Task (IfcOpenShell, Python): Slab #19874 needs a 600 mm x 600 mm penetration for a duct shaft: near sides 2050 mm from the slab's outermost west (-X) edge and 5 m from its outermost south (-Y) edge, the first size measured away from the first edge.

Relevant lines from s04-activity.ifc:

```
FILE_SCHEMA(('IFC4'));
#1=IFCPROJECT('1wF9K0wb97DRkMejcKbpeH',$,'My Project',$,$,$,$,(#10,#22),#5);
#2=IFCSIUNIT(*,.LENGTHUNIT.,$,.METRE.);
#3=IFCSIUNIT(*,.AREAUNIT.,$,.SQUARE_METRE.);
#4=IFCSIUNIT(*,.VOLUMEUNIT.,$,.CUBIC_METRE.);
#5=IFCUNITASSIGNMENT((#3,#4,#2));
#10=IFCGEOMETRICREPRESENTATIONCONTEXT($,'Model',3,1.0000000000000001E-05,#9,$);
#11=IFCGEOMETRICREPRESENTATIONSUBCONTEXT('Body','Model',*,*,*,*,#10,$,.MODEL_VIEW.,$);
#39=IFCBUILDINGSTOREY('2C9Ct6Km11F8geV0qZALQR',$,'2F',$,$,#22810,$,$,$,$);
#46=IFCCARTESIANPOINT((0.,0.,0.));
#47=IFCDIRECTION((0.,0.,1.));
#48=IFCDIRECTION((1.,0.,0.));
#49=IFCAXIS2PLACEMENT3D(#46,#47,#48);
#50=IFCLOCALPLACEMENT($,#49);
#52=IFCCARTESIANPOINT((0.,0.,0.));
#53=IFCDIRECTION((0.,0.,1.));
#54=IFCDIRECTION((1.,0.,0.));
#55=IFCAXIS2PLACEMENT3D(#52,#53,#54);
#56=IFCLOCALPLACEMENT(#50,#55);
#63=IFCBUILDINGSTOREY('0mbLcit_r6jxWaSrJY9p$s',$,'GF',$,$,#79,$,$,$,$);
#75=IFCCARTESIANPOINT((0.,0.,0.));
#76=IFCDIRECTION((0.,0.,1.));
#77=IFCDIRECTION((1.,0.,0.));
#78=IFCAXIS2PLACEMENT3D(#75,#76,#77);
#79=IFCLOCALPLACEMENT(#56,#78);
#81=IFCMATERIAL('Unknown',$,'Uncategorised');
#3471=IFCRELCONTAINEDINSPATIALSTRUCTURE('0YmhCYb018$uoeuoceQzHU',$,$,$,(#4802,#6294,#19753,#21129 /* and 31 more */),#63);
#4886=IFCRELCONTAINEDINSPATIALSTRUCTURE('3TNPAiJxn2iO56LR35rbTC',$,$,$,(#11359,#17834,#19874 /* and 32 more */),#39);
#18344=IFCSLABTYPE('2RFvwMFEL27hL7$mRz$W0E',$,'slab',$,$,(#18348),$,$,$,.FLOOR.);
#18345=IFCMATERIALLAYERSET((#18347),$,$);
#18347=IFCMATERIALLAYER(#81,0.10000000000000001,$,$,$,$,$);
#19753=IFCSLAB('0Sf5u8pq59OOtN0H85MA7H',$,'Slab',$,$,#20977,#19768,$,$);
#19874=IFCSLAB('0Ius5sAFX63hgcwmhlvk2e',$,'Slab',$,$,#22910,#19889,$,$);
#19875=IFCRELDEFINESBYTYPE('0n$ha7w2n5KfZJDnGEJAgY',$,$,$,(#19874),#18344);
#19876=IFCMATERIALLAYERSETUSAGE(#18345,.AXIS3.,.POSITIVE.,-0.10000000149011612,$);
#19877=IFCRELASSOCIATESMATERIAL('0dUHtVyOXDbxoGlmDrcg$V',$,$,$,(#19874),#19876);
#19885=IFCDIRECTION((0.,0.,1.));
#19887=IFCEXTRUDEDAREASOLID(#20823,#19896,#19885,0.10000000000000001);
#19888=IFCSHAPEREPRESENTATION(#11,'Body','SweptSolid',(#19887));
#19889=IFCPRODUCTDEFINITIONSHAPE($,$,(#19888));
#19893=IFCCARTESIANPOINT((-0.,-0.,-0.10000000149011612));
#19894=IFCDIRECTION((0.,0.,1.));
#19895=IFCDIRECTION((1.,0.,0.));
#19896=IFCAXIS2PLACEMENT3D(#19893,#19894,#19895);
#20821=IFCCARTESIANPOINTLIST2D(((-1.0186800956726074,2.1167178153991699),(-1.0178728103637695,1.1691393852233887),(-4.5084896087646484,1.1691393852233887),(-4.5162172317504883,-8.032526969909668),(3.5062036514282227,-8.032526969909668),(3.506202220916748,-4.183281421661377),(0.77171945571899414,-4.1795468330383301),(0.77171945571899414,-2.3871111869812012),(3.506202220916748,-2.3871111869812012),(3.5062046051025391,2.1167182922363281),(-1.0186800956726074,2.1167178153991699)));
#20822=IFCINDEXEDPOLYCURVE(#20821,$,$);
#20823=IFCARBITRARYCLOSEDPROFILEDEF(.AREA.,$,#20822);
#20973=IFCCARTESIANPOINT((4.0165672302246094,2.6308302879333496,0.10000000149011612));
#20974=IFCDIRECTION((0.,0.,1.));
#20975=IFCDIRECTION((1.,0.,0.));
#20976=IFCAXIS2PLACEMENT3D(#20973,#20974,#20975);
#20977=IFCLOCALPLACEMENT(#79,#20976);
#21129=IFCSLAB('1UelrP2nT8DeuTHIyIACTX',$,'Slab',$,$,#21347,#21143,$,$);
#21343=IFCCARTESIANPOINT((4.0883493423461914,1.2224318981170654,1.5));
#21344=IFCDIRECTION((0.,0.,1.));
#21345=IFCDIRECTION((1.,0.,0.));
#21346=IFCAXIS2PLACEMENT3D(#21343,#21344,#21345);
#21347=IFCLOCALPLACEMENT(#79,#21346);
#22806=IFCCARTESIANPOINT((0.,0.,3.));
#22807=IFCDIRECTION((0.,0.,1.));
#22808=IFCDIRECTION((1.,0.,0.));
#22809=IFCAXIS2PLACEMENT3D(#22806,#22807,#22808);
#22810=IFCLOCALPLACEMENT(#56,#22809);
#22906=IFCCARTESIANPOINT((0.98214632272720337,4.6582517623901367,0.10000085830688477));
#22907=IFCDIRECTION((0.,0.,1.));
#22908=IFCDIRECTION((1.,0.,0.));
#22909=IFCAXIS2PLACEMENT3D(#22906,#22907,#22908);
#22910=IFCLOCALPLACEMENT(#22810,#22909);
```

```python
import numpy as np
import ifcopenshell
import ifcopenshell.api.feature
import ifcopenshell.api.geometry
import ifcopenshell.api.root
import ifcopenshell.geom
import ifcopenshell.util.placement
import ifcopenshell.util.representation
import ifcopenshell.util.shape
import ifcopenshell.util.unit

model = ifcopenshell.open("s04-activity.ifc")
unit_scale = ifcopenshell.util.unit.calculate_unit_scale(model)
settings = ifcopenshell.geom.settings()


def volume(element):
    """Net volume in cubic metres, openings subtracted."""
    shape = ifcopenshell.geom.create_shape(settings, element)
    return ifcopenshell.util.shape.get_volume(shape.geometry)


slab = model.by_guid("0Ius5sAFX63hgcwmhlvk2e")
before = volume(slab)

# Extent in the slab's own axes, in metres. The edges named are its -X and -Y sides.
slab_shape = ifcopenshell.geom.create_shape(settings, slab)
vertices = ifcopenshell.util.shape.get_vertices(slab_shape.geometry)
x_min, y_min, bottom = vertices.min(axis=0)
top = vertices[:, 2].max()

opening = ifcopenshell.api.root.create_entity(model, ifc_class="IfcOpeningElement", name="Duct shaft opening", predefined_type="OPENING")
context = ifcopenshell.util.representation.get_context(model, "Model", "Body", "MODEL_VIEW")
width, depth = 0.6, 0.6
outline = [(0.0, 0.0), (width, 0.0), (width, depth), (0.0, depth), (0.0, 0.0)]
# Overshoot both faces by 50 mm so the cut is clean.
shape = ifcopenshell.api.geometry.add_slab_representation(
    model, context=context, depth=top - bottom + 0.1, polyline=outline
)
ifcopenshell.api.geometry.assign_representation(model, product=opening, representation=shape)

matrix = ifcopenshell.util.placement.get_local_placement(slab.ObjectPlacement)
matrix[:, 3] = matrix @ np.append(np.array([x_min + 2.05, y_min + 5, bottom - 0.05]) / unit_scale, 1.0)
ifcopenshell.api.geometry.edit_object_placement(model, product=opening, matrix=matrix, is_si=False)
ifcopenshell.api.feature.add_feature(model, feature=opening, element=slab)

after = volume(slab)

print(f"slab volume {before:.3f} -> {after:.3f} m3")

model.write("s04-activity_updated.ifc")
```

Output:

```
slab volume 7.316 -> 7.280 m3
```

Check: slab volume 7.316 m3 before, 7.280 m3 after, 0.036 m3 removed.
